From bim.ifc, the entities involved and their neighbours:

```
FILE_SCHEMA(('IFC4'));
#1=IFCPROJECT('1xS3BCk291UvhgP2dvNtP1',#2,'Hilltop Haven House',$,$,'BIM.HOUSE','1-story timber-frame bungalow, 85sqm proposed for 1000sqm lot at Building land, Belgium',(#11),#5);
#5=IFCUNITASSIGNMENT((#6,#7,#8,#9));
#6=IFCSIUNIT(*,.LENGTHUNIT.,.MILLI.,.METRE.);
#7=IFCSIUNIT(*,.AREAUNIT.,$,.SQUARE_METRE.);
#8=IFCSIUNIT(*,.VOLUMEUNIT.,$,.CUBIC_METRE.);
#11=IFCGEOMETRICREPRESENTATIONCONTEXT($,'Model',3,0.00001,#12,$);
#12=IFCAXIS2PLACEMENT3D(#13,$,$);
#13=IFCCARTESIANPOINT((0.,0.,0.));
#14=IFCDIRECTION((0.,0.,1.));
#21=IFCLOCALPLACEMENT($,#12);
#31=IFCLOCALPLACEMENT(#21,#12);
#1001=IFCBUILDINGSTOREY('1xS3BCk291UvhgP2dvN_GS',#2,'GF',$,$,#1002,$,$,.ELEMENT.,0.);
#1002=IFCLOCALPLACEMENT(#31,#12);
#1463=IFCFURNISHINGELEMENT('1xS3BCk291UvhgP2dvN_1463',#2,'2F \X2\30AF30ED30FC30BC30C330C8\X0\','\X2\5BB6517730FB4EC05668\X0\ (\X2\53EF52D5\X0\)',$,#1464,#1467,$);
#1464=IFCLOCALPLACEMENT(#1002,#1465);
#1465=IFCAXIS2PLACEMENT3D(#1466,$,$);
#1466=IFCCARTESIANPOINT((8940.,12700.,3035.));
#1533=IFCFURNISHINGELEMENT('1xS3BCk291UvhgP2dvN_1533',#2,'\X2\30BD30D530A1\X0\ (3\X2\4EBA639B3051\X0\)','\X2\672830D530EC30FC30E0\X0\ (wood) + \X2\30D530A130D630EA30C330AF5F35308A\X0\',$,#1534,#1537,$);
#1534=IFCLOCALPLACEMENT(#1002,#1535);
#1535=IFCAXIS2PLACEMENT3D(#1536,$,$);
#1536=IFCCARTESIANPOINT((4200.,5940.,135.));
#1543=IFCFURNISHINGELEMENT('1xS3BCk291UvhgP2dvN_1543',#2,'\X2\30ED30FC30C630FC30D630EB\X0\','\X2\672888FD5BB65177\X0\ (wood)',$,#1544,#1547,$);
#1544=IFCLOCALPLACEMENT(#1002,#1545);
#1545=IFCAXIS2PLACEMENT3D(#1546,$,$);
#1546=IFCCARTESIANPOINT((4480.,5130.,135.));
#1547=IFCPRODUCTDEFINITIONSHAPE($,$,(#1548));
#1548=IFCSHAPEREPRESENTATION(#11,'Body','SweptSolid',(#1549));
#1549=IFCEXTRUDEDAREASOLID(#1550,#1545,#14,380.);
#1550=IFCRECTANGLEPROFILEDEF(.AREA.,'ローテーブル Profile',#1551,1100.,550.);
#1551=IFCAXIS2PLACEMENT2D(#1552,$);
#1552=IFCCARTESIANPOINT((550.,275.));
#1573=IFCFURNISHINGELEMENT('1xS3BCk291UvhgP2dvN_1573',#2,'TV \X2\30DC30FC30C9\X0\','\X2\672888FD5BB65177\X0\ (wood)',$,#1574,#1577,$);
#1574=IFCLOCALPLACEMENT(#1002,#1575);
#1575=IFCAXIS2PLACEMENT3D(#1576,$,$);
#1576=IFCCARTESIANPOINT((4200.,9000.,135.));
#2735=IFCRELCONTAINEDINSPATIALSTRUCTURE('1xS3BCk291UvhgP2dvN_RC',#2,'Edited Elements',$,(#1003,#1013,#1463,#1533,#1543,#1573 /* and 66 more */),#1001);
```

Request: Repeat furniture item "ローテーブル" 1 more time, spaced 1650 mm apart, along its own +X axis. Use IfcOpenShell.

```python
import ifcopenshell
import ifcopenshell.api.geometry
import ifcopenshell.api.root
import ifcopenshell.util.element
import ifcopenshell.util.placement
import ifcopenshell.util.unit

model = ifcopenshell.open("bim.ifc")
unit_scale = ifcopenshell.util.unit.calculate_unit_scale(model)


def reuse_history(source, copy):
    """copy_class also copies each property set's owner history, people and application; keep the originals."""
    for rel in copy.IsDefinedBy:
        if rel.is_a("IfcRelDefinesByProperties") and (history := rel.RelatingPropertyDefinition.OwnerHistory):
            rel.RelatingPropertyDefinition.OwnerHistory = source.OwnerHistory
            ifcopenshell.util.element.remove_deep2(model, history)


source = model.by_guid("1xS3BCk291UvhgP2dvN_1543")
base = ifcopenshell.util.placement.get_local_placement(source.ObjectPlacement)
step = base[:3, 0] * 1.65 / unit_scale

for i in range(1, 2):
    copy = ifcopenshell.api.root.copy_class(model, product=source)
    copy.Representation = ifcopenshell.util.element.copy_deep(
        model, source.Representation, exclude=["IfcGeometricRepresentationContext", "IfcRepresentationMap"]
    )
    reuse_history(source, copy)
    matrix = base.copy()
    matrix[:3, 3] += i * step
    print("added at", matrix[:3, 3].round(3) + 0.0)
    ifcopenshell.api.geometry.edit_object_placement(model, product=copy, matrix=matrix, is_si=False)

model.write("bim_edited.ifc")
```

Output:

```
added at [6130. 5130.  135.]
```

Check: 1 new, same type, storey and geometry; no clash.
